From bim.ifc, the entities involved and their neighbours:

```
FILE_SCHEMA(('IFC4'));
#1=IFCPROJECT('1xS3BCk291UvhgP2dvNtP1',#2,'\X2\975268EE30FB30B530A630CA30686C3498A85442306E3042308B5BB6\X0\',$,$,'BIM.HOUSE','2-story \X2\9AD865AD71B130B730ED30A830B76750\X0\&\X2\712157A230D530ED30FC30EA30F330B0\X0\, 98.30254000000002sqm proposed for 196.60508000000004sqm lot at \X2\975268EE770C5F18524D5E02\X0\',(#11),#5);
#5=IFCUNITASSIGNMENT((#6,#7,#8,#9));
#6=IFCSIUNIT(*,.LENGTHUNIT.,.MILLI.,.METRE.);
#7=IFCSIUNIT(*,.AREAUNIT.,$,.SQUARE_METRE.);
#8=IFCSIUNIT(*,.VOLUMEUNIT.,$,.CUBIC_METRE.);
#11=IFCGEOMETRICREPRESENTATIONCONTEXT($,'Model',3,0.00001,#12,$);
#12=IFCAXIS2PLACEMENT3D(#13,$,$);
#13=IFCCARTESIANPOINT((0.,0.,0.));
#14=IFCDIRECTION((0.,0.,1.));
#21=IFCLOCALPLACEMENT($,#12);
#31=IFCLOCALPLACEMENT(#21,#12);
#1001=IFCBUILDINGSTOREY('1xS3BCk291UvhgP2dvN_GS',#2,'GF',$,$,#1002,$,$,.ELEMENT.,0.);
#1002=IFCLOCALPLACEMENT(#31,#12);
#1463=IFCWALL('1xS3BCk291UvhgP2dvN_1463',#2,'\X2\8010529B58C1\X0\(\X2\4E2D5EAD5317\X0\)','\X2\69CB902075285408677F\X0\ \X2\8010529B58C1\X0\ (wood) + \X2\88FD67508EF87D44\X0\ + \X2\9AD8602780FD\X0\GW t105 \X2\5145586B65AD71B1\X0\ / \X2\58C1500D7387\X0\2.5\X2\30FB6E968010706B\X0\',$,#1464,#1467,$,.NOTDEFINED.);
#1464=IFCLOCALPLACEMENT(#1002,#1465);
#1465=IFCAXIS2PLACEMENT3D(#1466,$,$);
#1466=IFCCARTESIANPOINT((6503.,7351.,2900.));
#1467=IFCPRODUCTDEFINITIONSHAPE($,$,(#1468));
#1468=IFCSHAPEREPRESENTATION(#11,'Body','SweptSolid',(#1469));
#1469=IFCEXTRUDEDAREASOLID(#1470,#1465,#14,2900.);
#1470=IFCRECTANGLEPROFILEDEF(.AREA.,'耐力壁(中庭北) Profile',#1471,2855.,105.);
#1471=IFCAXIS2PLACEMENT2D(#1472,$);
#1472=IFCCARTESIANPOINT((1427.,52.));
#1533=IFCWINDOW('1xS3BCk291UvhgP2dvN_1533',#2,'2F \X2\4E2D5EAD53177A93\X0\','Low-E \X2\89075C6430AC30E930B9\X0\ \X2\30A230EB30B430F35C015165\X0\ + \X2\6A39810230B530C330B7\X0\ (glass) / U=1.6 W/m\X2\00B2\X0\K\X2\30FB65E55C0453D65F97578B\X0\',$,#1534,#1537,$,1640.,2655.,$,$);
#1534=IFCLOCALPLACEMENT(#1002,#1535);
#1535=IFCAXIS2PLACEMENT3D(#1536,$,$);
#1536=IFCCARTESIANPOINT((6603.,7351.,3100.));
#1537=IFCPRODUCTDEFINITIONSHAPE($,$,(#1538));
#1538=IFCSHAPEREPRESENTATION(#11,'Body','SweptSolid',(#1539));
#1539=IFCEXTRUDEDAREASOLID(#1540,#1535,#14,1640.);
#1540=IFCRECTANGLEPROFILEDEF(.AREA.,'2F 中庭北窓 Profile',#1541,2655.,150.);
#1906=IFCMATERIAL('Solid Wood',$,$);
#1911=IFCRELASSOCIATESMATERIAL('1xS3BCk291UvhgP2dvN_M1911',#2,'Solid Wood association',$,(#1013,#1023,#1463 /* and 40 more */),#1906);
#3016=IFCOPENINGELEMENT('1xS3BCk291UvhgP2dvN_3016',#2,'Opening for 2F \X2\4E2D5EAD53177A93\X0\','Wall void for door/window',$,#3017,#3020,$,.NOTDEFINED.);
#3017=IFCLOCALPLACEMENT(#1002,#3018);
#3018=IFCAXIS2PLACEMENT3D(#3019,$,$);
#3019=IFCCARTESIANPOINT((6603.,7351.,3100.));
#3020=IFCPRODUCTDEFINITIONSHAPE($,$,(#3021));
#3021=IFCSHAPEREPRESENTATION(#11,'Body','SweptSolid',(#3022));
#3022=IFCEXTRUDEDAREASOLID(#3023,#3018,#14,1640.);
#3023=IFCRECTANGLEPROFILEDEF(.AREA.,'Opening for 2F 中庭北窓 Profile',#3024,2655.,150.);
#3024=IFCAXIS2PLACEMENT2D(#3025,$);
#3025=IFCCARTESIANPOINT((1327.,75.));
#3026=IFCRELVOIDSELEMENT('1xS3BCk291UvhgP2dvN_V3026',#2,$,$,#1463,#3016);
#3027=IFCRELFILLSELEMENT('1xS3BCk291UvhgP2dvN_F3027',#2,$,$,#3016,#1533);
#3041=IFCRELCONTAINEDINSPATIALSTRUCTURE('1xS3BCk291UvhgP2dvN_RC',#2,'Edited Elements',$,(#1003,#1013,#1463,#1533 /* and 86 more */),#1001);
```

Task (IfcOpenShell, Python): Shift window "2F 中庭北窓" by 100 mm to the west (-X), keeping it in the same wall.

```python
import ifcopenshell
import ifcopenshell.api.geometry
import ifcopenshell.util.placement
import ifcopenshell.util.unit

model = ifcopenshell.open("bim.ifc")
unit_scale = ifcopenshell.util.unit.calculate_unit_scale(model)

window = model.by_guid("1xS3BCk291UvhgP2dvN_1533")
opening = window.FillsVoids[0].RelatingOpeningElement
wall = opening.VoidsElements[0].RelatingBuildingElement

wall_matrix = ifcopenshell.util.placement.get_local_placement(wall.ObjectPlacement)
shift = wall_matrix[:3, 0] * -0.1 / unit_scale
before = ifcopenshell.util.placement.get_local_placement(window.ObjectPlacement)[:3, 3].copy()

# The window is not placed relative to its opening, so move both.
for product in (opening, window):
    matrix = ifcopenshell.util.placement.get_local_placement(product.ObjectPlacement)
    matrix[:3, 3] += shift
    ifcopenshell.api.geometry.edit_object_placement(model, product=product, matrix=matrix, is_si=False)

after = ifcopenshell.util.placement.get_local_placement(window.ObjectPlacement)[:3, 3]
print("window moved by", (after - before).round(3) + 0.0)

model.write("bim_rev.ifc")
```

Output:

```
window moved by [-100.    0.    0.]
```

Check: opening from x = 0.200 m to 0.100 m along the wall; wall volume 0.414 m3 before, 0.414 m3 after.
